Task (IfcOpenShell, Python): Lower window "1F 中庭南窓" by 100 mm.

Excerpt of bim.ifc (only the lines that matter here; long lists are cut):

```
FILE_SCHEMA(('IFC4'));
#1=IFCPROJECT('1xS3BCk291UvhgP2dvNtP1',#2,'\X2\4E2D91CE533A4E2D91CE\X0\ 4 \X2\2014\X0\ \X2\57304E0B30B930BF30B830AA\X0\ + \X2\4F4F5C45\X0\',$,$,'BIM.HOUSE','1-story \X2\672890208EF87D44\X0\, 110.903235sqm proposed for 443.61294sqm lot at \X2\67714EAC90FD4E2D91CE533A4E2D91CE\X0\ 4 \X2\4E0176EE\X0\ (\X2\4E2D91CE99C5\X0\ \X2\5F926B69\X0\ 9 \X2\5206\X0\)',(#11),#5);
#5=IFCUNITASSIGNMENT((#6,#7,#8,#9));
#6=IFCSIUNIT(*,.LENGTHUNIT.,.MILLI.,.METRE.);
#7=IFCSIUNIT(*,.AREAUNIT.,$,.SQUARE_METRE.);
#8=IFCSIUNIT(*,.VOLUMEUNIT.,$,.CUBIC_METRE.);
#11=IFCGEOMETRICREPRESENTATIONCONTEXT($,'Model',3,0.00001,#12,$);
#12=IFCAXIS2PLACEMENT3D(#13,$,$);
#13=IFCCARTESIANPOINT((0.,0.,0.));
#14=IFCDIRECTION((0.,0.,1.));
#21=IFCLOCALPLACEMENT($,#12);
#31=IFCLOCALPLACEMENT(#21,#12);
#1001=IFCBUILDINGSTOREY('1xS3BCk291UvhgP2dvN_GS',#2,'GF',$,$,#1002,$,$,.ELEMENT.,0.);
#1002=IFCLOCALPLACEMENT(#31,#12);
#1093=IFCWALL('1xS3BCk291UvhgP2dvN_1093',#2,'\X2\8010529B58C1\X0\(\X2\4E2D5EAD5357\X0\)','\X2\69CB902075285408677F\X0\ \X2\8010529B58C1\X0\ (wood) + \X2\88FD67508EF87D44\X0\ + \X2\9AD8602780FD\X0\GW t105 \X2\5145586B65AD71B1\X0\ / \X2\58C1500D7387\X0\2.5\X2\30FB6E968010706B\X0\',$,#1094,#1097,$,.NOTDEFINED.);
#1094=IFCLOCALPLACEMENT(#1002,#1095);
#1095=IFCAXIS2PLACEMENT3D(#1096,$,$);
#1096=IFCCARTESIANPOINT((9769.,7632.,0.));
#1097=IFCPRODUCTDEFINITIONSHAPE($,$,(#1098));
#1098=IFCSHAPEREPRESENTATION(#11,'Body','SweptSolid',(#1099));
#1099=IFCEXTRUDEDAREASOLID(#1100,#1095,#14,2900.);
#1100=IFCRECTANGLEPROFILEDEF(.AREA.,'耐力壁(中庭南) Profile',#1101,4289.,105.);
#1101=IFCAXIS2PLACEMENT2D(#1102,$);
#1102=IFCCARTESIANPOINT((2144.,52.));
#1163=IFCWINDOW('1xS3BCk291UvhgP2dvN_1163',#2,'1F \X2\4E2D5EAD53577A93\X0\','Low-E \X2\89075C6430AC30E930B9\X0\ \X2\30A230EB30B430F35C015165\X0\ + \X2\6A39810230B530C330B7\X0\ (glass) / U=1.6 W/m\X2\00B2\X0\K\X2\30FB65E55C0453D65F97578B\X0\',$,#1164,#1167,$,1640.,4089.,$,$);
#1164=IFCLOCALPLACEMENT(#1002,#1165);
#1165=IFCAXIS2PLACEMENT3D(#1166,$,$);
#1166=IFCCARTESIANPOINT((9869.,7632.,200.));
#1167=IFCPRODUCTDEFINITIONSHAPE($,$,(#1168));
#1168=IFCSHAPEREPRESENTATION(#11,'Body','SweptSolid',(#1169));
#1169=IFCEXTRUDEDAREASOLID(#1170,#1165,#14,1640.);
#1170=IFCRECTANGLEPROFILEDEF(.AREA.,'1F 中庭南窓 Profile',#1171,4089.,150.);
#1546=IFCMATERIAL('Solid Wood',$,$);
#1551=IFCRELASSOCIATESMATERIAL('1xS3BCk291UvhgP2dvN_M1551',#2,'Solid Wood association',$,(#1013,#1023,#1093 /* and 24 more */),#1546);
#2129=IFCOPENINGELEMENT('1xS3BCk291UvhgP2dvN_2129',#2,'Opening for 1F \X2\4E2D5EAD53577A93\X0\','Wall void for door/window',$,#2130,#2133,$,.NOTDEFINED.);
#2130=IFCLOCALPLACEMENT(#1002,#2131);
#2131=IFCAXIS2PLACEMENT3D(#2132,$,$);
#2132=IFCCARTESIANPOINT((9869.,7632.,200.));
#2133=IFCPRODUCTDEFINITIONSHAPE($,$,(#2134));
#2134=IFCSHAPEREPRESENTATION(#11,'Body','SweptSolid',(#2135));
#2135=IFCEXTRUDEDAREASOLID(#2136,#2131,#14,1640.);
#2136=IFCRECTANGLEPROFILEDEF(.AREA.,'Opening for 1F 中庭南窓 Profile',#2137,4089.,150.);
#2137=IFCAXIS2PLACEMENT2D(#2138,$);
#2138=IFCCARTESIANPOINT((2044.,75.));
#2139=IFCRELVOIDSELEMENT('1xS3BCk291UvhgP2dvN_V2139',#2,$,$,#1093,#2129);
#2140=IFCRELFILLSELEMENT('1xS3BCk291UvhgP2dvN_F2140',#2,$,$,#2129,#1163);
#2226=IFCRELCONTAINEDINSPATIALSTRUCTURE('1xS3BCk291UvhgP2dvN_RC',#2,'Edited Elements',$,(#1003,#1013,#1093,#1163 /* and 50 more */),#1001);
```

```python
import numpy as np
import ifcopenshell
import ifcopenshell.api.geometry
import ifcopenshell.util.placement
import ifcopenshell.util.unit

model = ifcopenshell.open("bim.ifc")
unit_scale = ifcopenshell.util.unit.calculate_unit_scale(model)

window = model.by_guid("1xS3BCk291UvhgP2dvN_1163")
opening = window.FillsVoids[0].RelatingOpeningElement
dz = -100.0

shift = np.array([0.0, 0.0, dz])
# The window is not placed relative to its opening, so move both.
for product in (opening, window):
    matrix = ifcopenshell.util.placement.get_local_placement(product.ObjectPlacement)
    matrix[:3, 3] += shift
    ifcopenshell.api.geometry.edit_object_placement(model, product=product, matrix=matrix, is_si=False)

print(f"moved by {dz * unit_scale:+.3f} m")

model.write("bim_updated.ifc")
```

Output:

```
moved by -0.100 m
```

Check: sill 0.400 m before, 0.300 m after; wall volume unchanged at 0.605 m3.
